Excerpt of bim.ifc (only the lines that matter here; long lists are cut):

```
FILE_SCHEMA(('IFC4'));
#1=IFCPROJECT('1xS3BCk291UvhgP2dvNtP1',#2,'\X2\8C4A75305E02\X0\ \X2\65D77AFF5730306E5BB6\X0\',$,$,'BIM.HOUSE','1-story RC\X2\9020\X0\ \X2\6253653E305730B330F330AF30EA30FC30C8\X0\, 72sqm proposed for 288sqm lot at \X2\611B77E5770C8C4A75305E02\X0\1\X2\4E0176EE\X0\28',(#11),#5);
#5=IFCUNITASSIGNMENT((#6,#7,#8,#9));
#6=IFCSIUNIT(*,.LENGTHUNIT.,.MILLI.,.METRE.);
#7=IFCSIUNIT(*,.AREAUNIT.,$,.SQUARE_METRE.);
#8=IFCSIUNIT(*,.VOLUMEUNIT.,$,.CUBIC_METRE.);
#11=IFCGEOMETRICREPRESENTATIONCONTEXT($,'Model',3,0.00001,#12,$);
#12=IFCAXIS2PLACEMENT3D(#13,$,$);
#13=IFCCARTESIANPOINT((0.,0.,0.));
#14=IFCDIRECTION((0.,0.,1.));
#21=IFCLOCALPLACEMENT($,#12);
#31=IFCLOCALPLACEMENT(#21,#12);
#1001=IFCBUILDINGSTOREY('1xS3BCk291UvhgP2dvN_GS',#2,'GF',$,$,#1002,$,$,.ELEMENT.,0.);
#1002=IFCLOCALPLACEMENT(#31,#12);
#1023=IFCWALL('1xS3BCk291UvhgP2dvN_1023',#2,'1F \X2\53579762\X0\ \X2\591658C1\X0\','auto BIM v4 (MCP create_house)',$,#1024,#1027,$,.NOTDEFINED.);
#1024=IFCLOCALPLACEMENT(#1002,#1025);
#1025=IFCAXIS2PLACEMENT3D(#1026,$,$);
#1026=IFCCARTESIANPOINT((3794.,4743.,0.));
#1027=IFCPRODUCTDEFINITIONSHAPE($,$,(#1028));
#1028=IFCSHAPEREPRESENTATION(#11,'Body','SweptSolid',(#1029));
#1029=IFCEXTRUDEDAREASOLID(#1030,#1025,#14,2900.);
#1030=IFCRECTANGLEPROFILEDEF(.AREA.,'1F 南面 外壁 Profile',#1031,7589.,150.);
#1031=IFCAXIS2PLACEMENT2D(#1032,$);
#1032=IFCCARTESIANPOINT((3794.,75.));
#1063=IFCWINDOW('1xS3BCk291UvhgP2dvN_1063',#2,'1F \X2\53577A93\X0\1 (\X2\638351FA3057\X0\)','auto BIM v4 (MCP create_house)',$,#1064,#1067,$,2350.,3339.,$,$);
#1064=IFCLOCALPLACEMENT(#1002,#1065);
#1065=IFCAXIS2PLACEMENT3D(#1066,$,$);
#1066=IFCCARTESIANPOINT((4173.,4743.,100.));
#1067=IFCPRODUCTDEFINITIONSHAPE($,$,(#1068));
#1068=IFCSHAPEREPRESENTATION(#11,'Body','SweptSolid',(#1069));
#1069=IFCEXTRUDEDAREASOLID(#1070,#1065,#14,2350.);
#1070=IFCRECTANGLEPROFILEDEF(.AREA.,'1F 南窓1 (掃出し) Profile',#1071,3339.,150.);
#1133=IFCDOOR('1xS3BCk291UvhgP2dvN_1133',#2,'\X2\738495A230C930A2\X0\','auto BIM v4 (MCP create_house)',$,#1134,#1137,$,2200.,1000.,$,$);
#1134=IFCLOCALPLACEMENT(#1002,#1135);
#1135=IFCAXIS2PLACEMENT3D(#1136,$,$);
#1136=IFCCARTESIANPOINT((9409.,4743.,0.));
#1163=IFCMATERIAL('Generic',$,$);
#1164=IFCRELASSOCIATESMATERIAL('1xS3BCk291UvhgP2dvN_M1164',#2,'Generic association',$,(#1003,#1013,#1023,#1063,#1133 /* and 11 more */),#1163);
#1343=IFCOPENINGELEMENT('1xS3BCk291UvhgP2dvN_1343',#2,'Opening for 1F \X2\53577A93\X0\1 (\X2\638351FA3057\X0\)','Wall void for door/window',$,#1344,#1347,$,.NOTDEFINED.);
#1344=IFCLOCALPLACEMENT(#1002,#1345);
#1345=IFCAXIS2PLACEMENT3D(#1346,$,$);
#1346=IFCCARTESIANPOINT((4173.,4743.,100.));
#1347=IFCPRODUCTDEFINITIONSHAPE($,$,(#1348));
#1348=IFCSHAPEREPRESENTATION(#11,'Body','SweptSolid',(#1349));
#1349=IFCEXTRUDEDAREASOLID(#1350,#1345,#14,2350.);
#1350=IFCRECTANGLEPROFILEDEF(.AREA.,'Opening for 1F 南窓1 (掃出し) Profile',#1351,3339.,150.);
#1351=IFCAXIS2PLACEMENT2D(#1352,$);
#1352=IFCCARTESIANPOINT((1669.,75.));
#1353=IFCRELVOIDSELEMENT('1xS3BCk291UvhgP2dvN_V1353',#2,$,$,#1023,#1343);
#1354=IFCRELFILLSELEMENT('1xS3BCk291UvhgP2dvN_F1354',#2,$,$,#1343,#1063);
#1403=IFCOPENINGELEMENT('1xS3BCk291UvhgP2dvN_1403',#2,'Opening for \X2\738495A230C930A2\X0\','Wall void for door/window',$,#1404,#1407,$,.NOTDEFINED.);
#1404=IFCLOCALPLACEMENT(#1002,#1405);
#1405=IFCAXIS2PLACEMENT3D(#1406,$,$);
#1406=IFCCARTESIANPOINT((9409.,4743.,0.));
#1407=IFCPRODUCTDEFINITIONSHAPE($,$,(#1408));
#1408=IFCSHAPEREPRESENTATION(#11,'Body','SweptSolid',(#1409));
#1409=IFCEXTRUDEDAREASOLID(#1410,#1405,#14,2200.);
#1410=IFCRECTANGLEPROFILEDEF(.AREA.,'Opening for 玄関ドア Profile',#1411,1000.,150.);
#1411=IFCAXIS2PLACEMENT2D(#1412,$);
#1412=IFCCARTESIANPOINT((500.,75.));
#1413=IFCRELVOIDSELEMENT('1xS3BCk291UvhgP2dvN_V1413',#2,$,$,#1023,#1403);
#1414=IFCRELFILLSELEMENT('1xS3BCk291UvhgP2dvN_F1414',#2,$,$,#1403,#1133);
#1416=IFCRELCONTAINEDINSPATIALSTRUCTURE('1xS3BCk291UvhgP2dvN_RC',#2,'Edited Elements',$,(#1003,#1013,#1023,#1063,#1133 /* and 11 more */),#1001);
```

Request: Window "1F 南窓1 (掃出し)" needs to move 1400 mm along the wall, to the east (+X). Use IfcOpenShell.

```python
import ifcopenshell
import ifcopenshell.api.geometry
import ifcopenshell.util.placement
import ifcopenshell.util.unit

model = ifcopenshell.open("bim.ifc")
unit_scale = ifcopenshell.util.unit.calculate_unit_scale(model)

window = model.by_id(1063)
opening = window.FillsVoids[0].RelatingOpeningElement
wall = opening.VoidsElements[0].RelatingBuildingElement

wall_matrix = ifcopenshell.util.placement.get_local_placement(wall.ObjectPlacement)
shift = wall_matrix[:3, 0] * 1.4 / unit_scale
before = ifcopenshell.util.placement.get_local_placement(window.ObjectPlacement)[:3, 3].copy()

# The window is not placed relative to its opening, so move both.
for product in (opening, window):
    matrix = ifcopenshell.util.placement.get_local_placement(product.ObjectPlacement)
    matrix[:3, 3] += shift
    ifcopenshell.api.geometry.edit_object_placement(model, product=product, matrix=matrix, is_si=False)

after = ifcopenshell.util.placement.get_local_placement(window.ObjectPlacement)[:3, 3]
print("window moved by", (after - before).round(3) + 0.0)

model.write("bim-out.ifc")
```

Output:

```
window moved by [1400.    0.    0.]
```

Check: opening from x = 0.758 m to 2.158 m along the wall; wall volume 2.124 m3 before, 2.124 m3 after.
